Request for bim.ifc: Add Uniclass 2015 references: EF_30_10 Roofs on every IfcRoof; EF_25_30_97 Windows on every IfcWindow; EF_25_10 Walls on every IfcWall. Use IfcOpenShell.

First a look at what the model holds.

```python
import ifcopenshell

model = ifcopenshell.open("bim.ifc")
print(model.schema)
print("classifications:", [c.Name for c in model.by_type("IfcClassification")])
for ifc_class in ("IfcDoor", "IfcRoof", "IfcStair", "IfcWall", "IfcWindow"):
    print(ifc_class, len(model.by_type(ifc_class)))
```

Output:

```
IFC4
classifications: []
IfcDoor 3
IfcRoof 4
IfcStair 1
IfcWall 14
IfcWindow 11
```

```python
import ifcopenshell
import ifcopenshell.api.classification

model = ifcopenshell.open("bim.ifc")

system = ifcopenshell.api.classification.add_classification(model, classification="Uniclass 2015")

codes = {
    "IfcRoof": ("EF_30_10", "Roofs"),
    "IfcWindow": ("EF_25_30_97", "Windows"),
    "IfcWall": ("EF_25_10", "Walls"),
}
for ifc_class, (code, name) in codes.items():
    products = model.by_type(ifc_class)
    ifcopenshell.api.classification.add_reference(
        model, products=products, classification=system, identification=code, name=name
    )
    print(code, len(products))

model.write("bim_v2.ifc")
```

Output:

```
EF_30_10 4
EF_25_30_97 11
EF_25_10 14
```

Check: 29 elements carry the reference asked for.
